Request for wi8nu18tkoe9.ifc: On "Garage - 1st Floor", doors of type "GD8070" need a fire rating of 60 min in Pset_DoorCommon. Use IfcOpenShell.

First a look at what the model holds.

```python
import ifcopenshell
import ifcopenshell.util.element

model = ifcopenshell.open("wi8nu18tkoe9.ifc")
print(model.schema)
storey = next(s for s in model.by_type("IfcBuildingStorey") if s.Name == "Garage - 1st Floor")
doors = [e for e in ifcopenshell.util.element.get_decomposition(storey) if e.is_a("IfcDoor")]
seen = {}
for e in doors:
    element_type = ifcopenshell.util.element.get_type(e)
    key = (element_type.Name if element_type != e and element_type else None, ifcopenshell.util.element.get_pset(e, "Pset_DoorCommon", "FireRating"))
    seen[key] = seen.get(key, 0) + 1
for (name, value), count in sorted(seen.items(), key=str):
    print(count, "x", name, "|", value)
```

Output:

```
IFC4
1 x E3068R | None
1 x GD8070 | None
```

```python
import ifcopenshell
import ifcopenshell.api.pset
import ifcopenshell.util.element

model = ifcopenshell.open("wi8nu18tkoe9.ifc")

storey = next(s for s in model.by_type("IfcBuildingStorey") if s.Name == "Garage - 1st Floor")
doors = [e for e in ifcopenshell.util.element.get_decomposition(storey) if e.is_a("IfcDoor")]

count = 0
for e in doors:
    element_type = ifcopenshell.util.element.get_type(e)
    if element_type in (None, e) or element_type.Name != "GD8070":
        continue
    # add_pset returns the element's existing set when there is one.
    pset = ifcopenshell.api.pset.add_pset(model, product=e, name="Pset_DoorCommon")
    ifcopenshell.api.pset.edit_pset(model, pset=pset, properties={"FireRating": "60 min"})
    count += 1

print(count, "doors updated")

model.write("wi8nu18tkoe9_edited.ifc")
```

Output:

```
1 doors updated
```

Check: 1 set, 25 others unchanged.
